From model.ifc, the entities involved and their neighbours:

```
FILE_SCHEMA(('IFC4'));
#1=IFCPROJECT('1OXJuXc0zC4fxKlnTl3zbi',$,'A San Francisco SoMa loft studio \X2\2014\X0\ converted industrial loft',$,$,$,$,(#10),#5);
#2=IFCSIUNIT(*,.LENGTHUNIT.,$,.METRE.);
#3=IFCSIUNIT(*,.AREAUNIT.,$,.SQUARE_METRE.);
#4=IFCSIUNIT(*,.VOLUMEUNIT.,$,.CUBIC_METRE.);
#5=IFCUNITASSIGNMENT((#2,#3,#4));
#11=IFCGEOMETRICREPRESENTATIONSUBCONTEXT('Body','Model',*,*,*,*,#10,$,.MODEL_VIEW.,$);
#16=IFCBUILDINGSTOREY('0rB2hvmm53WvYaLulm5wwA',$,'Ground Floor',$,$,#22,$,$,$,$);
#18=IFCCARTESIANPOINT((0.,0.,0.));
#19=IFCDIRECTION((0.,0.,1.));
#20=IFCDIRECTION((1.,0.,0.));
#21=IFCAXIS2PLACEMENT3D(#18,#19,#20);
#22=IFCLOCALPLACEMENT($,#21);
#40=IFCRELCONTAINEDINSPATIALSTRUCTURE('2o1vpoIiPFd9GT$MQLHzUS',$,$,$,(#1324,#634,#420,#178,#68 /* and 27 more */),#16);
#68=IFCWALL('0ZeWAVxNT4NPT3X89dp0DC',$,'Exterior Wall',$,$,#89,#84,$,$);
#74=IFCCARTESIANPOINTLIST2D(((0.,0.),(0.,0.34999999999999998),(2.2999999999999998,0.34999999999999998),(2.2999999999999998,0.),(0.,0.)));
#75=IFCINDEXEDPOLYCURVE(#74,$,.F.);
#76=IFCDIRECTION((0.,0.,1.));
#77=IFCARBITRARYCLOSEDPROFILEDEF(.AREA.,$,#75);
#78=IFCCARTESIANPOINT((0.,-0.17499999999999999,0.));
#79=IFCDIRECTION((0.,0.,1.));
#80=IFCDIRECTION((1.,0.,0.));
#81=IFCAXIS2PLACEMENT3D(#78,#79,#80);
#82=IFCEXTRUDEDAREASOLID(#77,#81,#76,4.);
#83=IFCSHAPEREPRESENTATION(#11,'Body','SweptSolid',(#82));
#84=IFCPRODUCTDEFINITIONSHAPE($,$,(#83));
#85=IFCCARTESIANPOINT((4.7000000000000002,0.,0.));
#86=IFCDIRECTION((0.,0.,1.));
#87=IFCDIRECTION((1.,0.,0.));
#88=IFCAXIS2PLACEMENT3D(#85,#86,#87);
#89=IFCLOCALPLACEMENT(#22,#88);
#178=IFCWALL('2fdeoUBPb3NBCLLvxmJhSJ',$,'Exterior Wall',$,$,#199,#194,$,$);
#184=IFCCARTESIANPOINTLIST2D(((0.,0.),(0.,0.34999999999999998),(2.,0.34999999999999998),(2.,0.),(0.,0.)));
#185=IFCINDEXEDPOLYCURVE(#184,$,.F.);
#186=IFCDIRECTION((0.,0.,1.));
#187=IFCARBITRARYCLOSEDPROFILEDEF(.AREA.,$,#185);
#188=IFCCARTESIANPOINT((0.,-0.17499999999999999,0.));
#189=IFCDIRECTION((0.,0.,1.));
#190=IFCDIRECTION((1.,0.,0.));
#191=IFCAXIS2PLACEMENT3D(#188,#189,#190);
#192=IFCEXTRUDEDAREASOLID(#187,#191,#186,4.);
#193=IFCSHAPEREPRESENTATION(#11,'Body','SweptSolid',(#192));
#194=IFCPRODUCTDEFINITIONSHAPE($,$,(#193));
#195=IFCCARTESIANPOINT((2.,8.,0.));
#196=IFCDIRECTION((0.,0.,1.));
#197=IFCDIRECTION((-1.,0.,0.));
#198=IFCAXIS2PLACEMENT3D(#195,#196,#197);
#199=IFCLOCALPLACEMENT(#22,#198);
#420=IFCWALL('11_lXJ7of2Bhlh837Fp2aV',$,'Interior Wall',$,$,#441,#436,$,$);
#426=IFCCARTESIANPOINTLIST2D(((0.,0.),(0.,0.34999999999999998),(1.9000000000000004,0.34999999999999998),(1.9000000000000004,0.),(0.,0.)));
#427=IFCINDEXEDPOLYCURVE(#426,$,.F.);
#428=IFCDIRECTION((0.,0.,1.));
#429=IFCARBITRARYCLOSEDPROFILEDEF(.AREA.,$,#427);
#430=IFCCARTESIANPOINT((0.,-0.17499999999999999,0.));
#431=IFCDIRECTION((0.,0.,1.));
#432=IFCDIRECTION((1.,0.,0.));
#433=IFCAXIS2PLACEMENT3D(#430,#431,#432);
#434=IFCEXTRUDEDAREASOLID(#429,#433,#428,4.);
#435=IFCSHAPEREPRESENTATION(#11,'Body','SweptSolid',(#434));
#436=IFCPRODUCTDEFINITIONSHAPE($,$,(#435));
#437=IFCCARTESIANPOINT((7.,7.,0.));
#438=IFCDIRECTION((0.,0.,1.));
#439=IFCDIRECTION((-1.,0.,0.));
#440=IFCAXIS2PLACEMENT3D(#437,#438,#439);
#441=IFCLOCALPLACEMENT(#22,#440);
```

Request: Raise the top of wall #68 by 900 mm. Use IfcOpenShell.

```python
import ifcopenshell
import ifcopenshell.geom
import ifcopenshell.util.representation
import ifcopenshell.util.shape
import ifcopenshell.util.unit

model = ifcopenshell.open("model.ifc")
unit_scale = ifcopenshell.util.unit.calculate_unit_scale(model)
settings = ifcopenshell.geom.settings()


def volume(element):
    """Net volume in cubic metres, openings subtracted."""
    shape = ifcopenshell.geom.create_shape(settings, element)
    return ifcopenshell.util.shape.get_volume(shape.geometry)


wall = model.by_id(68)
before = volume(wall)

body = ifcopenshell.util.representation.get_representation(wall, "Model", "Body")
solid = body.Items[0]
old_height = solid.Depth
solid.Depth += 0.9 / unit_scale
after = volume(wall)

print(f"height {old_height:g} -> {solid.Depth:g}, volume {before:.3f} -> {after:.3f} m3")

model.write("model_updated.ifc")
```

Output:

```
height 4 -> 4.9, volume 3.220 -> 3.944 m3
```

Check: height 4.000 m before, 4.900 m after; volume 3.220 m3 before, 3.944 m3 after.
